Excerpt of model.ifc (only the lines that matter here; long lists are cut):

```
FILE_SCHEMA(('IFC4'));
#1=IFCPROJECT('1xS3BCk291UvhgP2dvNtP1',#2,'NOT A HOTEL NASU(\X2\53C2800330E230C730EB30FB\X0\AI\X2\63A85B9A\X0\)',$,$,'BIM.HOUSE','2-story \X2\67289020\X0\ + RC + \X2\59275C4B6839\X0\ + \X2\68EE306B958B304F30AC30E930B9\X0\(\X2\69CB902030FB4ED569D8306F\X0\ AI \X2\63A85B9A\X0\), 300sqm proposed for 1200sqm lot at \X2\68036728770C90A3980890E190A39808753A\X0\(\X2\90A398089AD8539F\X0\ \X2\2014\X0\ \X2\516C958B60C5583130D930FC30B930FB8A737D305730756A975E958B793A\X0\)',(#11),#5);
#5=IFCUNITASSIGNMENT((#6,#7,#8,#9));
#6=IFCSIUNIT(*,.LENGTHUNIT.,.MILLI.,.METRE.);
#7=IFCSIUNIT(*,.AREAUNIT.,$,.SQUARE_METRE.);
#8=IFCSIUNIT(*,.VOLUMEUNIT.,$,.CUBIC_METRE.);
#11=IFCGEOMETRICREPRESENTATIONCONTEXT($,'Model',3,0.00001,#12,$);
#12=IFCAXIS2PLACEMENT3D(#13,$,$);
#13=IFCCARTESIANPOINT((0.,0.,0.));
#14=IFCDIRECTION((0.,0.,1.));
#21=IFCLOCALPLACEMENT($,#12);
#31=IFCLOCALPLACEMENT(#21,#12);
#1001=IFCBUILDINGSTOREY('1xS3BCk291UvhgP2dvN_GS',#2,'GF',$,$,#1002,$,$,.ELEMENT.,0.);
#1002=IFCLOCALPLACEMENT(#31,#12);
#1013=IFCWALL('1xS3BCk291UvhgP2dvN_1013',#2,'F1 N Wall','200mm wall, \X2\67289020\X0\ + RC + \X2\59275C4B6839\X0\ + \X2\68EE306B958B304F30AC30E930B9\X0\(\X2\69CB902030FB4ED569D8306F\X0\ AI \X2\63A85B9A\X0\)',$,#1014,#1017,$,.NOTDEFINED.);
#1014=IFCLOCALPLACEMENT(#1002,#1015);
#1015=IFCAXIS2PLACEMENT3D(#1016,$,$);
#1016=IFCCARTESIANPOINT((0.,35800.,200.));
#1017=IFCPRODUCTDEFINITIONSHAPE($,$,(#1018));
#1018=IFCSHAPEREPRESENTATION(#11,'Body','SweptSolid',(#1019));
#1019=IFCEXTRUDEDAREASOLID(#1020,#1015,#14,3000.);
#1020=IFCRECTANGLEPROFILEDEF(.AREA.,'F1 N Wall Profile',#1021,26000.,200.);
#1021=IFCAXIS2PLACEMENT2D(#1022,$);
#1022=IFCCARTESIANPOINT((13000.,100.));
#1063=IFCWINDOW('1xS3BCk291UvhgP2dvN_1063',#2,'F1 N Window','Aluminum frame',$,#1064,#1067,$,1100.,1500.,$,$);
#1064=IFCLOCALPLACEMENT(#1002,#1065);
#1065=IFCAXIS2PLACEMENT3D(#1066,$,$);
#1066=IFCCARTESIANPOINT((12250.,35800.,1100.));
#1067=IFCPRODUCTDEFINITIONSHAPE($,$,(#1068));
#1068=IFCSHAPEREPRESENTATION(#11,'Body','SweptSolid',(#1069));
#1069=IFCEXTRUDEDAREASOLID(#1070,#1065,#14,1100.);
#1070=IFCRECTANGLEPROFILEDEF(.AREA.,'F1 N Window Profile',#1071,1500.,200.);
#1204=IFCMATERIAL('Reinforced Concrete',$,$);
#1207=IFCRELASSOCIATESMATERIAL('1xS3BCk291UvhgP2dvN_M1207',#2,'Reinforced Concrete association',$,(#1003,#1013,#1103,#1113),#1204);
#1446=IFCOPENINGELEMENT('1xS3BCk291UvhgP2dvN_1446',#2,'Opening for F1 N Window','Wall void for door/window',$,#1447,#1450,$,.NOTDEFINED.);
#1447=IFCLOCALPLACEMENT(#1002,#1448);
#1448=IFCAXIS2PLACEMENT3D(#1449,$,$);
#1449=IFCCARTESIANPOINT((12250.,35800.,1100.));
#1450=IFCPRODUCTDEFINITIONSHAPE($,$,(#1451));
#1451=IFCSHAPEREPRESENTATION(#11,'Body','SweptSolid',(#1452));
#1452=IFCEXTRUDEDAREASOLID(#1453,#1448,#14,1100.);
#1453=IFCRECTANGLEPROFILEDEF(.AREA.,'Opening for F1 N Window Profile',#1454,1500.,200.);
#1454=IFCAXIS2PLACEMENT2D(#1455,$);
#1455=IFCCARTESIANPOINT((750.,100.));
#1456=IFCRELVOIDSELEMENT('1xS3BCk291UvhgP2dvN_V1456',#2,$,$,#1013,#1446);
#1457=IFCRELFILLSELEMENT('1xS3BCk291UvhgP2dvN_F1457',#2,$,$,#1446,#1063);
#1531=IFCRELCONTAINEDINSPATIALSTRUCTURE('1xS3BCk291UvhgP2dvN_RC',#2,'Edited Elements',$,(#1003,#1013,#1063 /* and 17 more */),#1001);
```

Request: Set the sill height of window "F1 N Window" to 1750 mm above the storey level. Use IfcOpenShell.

```python
import numpy as np
import ifcopenshell
import ifcopenshell.api.geometry
import ifcopenshell.geom
import ifcopenshell.util.element
import ifcopenshell.util.placement
import ifcopenshell.util.shape
import ifcopenshell.util.unit

model = ifcopenshell.open("model.ifc")
unit_scale = ifcopenshell.util.unit.calculate_unit_scale(model)

window = model.by_guid("1xS3BCk291UvhgP2dvN_1063")
opening = window.FillsVoids[0].RelatingOpeningElement
storey = ifcopenshell.util.element.get_container(window, ifc_class="IfcBuildingStorey")
level = ifcopenshell.util.placement.get_local_placement(storey.ObjectPlacement)[2, 3]

# The opening's origin need not be at the sill, so measure its lowest point.
shape = ifcopenshell.geom.create_shape(ifcopenshell.geom.settings(), opening)
bottom = ifcopenshell.util.shape.get_shape_bottom_elevation(shape, shape.geometry) / unit_scale
dz = level + 1.75 / unit_scale - bottom

shift = np.array([0.0, 0.0, dz])
# The window is not placed relative to its opening, so move both.
for product in (opening, window):
    matrix = ifcopenshell.util.placement.get_local_placement(product.ObjectPlacement)
    matrix[:3, 3] += shift
    ifcopenshell.api.geometry.edit_object_placement(model, product=product, matrix=matrix, is_si=False)

print(f"moved by {dz * unit_scale:+.3f} m")

model.write("model_rev.ifc")
```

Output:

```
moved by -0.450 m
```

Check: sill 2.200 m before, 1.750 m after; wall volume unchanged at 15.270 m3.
